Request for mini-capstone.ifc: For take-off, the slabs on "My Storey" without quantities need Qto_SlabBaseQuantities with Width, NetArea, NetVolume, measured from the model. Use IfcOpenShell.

First a look at what the model holds.

```python
import ifcopenshell
import ifcopenshell.util.element
import ifcopenshell.util.unit

model = ifcopenshell.open("mini-capstone.ifc")
print(model.schema)
for unit_type in ("LENGTHUNIT", "AREAUNIT", "VOLUMEUNIT"):
    print(unit_type, ifcopenshell.util.unit.calculate_unit_scale(model, unit_type))
storey = next(s for s in model.by_type("IfcBuildingStorey") if s.Name == "My Storey")
slabs = [e for e in ifcopenshell.util.element.get_decomposition(storey) if e.is_a("IfcSlab")]
for e in sorted(slabs, key=lambda e: e.id()):
    print(e.id(), e.is_a(), e.Name, list(ifcopenshell.util.element.get_psets(e, qtos_only=True)), sep=" | ")
```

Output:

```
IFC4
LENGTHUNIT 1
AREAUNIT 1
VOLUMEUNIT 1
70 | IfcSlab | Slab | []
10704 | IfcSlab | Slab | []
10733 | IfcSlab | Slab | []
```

```python
import ifcopenshell
import ifcopenshell.api.pset
import ifcopenshell.geom
import ifcopenshell.util.element
import ifcopenshell.util.shape
import ifcopenshell.util.unit

model = ifcopenshell.open("mini-capstone.ifc")
unit_scale = ifcopenshell.util.unit.calculate_unit_scale(model)
area_scale = ifcopenshell.util.unit.calculate_unit_scale(model, "AREAUNIT")
volume_scale = ifcopenshell.util.unit.calculate_unit_scale(model, "VOLUMEUNIT")
settings = ifcopenshell.geom.settings()

storey = next(s for s in model.by_type("IfcBuildingStorey") if s.Name == "My Storey")
slabs = [e for e in ifcopenshell.util.element.get_decomposition(storey) if e.is_a("IfcSlab")]

for e in sorted(slabs, key=lambda e: e.id()):
    if ifcopenshell.util.element.get_psets(e, qtos_only=True, should_inherit=False):
        continue
    # Geometry comes back in metres, in the element's own axes.
    shape = ifcopenshell.geom.create_shape(settings, e)
    values = {
        "Width": ifcopenshell.util.shape.get_z(shape.geometry) / unit_scale,
        "NetArea": ifcopenshell.util.shape.get_footprint_area(shape.geometry) / area_scale,
        "NetVolume": ifcopenshell.util.shape.get_volume(shape.geometry) / volume_scale,
    }
    qto = ifcopenshell.api.pset.add_qto(model, product=e, name="Qto_SlabBaseQuantities")
    ifcopenshell.api.pset.edit_qto(model, qto=qto, properties=values)
    print(e.id(), {k: round(v, 3) for k, v in values.items()})

model.write("mini-capstone_v2.ifc")
```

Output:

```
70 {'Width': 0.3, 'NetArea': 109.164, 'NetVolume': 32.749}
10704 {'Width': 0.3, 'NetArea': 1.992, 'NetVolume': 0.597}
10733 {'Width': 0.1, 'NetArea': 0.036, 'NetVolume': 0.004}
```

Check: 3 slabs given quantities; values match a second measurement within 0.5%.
